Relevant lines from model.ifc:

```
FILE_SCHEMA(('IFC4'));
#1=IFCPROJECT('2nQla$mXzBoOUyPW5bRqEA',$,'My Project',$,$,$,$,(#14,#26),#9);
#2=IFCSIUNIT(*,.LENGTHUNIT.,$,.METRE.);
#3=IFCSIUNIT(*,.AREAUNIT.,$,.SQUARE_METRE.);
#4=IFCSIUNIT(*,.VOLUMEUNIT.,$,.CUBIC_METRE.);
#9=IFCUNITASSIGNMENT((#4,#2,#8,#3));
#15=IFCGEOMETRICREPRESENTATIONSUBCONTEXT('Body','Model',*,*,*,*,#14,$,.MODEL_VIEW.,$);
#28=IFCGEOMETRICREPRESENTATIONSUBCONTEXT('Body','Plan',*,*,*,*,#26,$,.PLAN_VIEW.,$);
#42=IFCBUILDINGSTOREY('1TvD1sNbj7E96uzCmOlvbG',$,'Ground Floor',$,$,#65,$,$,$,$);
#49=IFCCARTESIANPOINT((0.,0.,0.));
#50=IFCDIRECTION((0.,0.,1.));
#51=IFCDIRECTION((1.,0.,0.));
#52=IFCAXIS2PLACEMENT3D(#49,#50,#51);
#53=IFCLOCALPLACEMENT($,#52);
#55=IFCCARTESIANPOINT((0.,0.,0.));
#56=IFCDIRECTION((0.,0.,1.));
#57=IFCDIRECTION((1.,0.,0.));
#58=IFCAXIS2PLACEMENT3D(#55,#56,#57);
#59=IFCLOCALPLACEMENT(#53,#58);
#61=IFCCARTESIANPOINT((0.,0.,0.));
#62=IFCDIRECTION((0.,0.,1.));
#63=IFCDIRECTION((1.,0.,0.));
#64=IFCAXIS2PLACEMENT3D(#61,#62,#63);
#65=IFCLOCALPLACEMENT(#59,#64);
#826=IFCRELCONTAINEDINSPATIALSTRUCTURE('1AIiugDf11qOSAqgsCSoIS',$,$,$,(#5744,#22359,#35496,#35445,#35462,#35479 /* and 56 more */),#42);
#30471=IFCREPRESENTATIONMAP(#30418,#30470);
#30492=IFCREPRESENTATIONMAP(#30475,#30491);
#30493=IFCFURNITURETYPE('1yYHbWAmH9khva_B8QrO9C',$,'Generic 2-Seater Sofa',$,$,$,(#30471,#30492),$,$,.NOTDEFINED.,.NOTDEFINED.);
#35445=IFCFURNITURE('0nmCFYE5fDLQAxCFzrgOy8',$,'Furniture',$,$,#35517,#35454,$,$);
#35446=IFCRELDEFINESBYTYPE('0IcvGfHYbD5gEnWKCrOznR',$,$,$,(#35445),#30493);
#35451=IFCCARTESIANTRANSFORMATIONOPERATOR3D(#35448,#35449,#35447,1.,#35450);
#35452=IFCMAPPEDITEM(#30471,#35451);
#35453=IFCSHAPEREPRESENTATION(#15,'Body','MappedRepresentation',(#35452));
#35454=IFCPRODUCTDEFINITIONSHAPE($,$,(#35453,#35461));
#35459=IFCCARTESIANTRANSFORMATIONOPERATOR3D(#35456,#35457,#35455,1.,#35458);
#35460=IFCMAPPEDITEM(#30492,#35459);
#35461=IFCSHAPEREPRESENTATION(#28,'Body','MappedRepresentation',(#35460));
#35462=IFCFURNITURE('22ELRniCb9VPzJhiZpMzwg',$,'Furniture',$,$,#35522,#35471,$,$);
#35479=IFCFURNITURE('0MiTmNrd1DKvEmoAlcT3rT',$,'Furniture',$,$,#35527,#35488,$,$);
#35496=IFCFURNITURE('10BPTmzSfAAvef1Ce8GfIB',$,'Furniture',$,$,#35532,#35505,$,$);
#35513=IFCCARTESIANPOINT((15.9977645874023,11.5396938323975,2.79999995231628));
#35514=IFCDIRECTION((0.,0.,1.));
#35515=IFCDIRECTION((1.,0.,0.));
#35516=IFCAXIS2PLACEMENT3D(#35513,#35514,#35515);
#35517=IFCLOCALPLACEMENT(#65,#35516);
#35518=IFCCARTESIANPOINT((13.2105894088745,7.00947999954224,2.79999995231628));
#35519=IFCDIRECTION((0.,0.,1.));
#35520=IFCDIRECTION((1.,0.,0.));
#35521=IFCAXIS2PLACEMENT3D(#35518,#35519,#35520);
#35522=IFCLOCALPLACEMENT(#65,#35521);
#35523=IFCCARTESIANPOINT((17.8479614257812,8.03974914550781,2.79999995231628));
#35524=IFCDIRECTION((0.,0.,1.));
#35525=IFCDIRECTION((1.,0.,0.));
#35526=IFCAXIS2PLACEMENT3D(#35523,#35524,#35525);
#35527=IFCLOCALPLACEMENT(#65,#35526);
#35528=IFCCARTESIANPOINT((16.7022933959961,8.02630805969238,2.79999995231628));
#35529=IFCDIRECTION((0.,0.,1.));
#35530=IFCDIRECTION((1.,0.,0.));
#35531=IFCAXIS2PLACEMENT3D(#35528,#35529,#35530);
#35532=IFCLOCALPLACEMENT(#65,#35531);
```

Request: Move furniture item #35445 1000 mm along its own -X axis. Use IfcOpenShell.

```python
import ifcopenshell
import ifcopenshell.api.geometry
import ifcopenshell.util.placement
import ifcopenshell.util.unit

model = ifcopenshell.open("model.ifc")
unit_scale = ifcopenshell.util.unit.calculate_unit_scale(model)

item = model.by_guid("0nmCFYE5fDLQAxCFzrgOy8")
matrix = ifcopenshell.util.placement.get_local_placement(item.ObjectPlacement)
matrix[:3, 3] -= matrix[:3, 0] * 1 / unit_scale
ifcopenshell.api.geometry.edit_object_placement(model, product=item, matrix=matrix, is_si=False)

print(ifcopenshell.util.placement.get_local_placement(item.ObjectPlacement).round(3) + 0.0)

model.write("model_edited.ifc")
```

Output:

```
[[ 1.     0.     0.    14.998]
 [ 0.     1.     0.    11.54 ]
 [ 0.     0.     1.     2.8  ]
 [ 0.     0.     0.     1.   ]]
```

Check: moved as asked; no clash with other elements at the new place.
